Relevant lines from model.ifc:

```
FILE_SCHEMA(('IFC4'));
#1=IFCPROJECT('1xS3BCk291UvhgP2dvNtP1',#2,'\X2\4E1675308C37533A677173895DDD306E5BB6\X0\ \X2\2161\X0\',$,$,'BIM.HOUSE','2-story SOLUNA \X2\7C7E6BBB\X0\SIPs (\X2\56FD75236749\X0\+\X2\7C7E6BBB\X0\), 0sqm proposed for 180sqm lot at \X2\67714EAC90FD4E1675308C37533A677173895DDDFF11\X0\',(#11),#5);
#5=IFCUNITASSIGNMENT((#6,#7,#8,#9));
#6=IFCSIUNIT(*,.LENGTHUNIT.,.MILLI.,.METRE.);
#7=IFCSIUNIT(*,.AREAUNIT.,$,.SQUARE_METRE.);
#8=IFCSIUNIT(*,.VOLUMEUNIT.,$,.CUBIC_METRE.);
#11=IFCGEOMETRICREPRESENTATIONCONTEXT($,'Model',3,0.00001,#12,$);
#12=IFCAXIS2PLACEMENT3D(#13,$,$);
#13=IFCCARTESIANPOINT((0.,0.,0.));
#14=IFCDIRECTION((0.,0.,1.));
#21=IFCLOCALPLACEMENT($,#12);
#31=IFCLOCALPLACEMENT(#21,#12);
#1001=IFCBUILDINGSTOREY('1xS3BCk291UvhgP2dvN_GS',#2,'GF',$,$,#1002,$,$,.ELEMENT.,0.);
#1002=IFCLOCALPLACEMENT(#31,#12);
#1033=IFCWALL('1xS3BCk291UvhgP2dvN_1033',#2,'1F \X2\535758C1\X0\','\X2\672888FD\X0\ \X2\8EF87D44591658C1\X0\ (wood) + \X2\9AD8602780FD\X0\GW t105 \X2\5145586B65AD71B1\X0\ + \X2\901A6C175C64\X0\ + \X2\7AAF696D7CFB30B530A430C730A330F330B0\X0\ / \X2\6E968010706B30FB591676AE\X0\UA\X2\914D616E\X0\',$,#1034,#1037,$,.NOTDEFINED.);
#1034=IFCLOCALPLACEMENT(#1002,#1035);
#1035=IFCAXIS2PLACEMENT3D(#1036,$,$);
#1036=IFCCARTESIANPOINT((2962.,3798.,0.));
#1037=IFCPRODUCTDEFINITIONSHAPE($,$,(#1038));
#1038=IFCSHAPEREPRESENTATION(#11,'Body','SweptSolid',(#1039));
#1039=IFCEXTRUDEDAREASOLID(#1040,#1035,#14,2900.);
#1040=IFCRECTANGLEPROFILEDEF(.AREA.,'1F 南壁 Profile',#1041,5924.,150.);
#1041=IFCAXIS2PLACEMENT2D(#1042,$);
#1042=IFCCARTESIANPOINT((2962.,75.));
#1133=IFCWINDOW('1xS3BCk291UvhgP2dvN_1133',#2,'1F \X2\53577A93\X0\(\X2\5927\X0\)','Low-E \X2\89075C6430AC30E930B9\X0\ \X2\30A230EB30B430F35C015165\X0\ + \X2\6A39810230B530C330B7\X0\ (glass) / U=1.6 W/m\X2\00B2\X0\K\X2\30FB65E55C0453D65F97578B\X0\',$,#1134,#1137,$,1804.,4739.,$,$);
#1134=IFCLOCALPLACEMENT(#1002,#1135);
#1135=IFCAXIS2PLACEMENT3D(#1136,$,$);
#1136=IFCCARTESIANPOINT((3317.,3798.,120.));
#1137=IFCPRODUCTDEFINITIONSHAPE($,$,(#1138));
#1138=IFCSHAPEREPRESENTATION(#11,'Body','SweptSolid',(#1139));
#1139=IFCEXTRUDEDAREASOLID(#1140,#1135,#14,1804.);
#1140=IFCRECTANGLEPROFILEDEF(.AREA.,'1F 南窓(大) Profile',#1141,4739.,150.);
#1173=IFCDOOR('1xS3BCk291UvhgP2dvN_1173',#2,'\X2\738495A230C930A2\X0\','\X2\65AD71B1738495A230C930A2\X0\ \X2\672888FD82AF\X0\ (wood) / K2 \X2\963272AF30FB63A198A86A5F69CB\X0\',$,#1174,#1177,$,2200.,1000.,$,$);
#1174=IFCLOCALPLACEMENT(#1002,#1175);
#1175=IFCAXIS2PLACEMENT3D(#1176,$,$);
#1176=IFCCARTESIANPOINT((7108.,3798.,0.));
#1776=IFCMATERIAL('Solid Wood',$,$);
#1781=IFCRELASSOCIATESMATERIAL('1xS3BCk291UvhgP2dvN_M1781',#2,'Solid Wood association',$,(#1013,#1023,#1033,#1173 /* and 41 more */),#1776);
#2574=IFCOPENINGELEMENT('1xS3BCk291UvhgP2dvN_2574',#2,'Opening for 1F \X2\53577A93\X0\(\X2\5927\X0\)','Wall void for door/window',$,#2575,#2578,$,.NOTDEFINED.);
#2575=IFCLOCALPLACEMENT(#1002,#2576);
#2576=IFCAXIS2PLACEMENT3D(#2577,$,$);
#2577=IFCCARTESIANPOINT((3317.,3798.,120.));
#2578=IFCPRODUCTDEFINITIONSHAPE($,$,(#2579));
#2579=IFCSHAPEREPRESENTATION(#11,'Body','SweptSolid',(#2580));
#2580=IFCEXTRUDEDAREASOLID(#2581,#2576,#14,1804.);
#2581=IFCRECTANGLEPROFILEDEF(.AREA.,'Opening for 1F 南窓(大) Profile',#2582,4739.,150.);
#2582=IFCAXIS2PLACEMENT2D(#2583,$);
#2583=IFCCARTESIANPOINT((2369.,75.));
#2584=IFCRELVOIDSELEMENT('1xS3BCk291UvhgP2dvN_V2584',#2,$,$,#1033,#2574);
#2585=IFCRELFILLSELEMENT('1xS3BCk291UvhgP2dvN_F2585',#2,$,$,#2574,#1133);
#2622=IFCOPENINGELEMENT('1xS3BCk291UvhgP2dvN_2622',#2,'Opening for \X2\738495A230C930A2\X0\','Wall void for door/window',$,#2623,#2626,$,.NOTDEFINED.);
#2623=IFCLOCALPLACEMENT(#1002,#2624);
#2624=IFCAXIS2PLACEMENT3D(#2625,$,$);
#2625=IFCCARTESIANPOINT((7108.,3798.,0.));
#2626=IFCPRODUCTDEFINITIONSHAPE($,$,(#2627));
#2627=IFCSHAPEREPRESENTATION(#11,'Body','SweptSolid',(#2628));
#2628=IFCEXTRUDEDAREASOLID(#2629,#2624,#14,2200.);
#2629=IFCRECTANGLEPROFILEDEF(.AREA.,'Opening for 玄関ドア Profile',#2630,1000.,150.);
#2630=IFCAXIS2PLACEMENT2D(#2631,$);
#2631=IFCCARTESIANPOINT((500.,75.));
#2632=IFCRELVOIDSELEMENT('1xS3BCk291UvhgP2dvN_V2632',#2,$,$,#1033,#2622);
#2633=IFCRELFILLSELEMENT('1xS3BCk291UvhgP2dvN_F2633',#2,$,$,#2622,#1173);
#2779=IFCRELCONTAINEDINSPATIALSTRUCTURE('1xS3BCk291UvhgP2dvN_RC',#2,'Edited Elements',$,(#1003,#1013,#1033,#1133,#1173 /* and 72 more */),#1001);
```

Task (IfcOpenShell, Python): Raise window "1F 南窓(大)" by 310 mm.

```python
import numpy as np
import ifcopenshell
import ifcopenshell.api.geometry
import ifcopenshell.util.placement
import ifcopenshell.util.unit

model = ifcopenshell.open("model.ifc")
unit_scale = ifcopenshell.util.unit.calculate_unit_scale(model)

window = model.by_guid("1xS3BCk291UvhgP2dvN_1133")
opening = window.FillsVoids[0].RelatingOpeningElement
dz = 0.31 / unit_scale

shift = np.array([0.0, 0.0, dz])
# The window is not placed relative to its opening, so move both.
for product in (opening, window):
    matrix = ifcopenshell.util.placement.get_local_placement(product.ObjectPlacement)
    matrix[:3, 3] += shift
    ifcopenshell.api.geometry.edit_object_placement(model, product=product, matrix=matrix, is_si=False)

print(f"moved by {dz * unit_scale:+.3f} m")

model.write("model_updated.ifc")
```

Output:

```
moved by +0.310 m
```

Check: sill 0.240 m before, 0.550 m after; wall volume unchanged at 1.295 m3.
